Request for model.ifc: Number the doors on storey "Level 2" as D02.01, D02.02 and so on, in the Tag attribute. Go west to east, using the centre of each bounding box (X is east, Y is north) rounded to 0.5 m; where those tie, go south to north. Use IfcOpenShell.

First a look at what the model holds.

```python
import ifcopenshell
import ifcopenshell.util.element
import ifcopenshell.util.placement

model = ifcopenshell.open("model.ifc")
print(model.schema)
storey = next(s for s in model.by_type("IfcBuildingStorey") if s.Name == "Level 2")
doors = [e for e in ifcopenshell.util.element.get_decomposition(storey) if e.is_a("IfcDoor")]
for e in sorted(doors, key=lambda e: e.id()):
    origin = ifcopenshell.util.placement.get_local_placement(e.ObjectPlacement)[:3, 3]
    print(e.id(), e.Tag, e.Name, origin.round(2) + 0.0, sep=" | ")
```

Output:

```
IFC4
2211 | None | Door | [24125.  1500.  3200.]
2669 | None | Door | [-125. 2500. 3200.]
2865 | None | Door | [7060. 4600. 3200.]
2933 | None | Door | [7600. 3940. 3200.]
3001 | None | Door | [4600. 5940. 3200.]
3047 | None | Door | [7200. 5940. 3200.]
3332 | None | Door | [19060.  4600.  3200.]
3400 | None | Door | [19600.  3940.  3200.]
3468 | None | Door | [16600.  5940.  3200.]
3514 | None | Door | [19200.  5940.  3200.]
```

```python
import ifcopenshell
import ifcopenshell.geom
import ifcopenshell.util.element
import ifcopenshell.util.shape

model = ifcopenshell.open("model.ifc")
settings = ifcopenshell.geom.settings()
settings.set("use-world-coords", True)


def centre(element):
    shape = ifcopenshell.geom.create_shape(settings, element)
    return ifcopenshell.util.shape.get_bbox_centroid(shape.geometry)


storey = next(s for s in model.by_type("IfcBuildingStorey") if s.Name == "Level 2")
doors = [e for e in ifcopenshell.util.element.get_decomposition(storey) if e.is_a("IfcDoor")]

# Insertion points can sit at a corner or the storey origin, so sort by the geometry (in metres).
centres = {e: centre(e) for e in doors}
doors.sort(key=lambda e: (round(centres[e][0] / 0.5), centres[e][1]))

for i, e in enumerate(doors, start=1):
    number = f"D02.{i:02d}"
    e.Tag = number
    print(e.id(), number)

model.write("model_v2.ifc")
```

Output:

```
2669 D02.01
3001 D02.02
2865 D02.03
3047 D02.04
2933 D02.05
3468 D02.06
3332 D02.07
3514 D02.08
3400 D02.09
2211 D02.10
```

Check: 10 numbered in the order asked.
